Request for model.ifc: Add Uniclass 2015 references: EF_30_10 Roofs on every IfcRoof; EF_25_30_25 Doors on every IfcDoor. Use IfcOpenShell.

First a look at what the model holds.

```python
import ifcopenshell

model = ifcopenshell.open("model.ifc")
print(model.schema)
print("classifications:", [c.Name for c in model.by_type("IfcClassification")])
for ifc_class in ("IfcDoor", "IfcRoof", "IfcStair", "IfcWall", "IfcWindow"):
    print(ifc_class, len(model.by_type(ifc_class)))
```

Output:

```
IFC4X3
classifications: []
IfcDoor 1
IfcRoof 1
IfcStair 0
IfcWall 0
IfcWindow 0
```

```python
import ifcopenshell
import ifcopenshell.api.classification

model = ifcopenshell.open("model.ifc")

system = ifcopenshell.api.classification.add_classification(model, classification="Uniclass 2015")

codes = {
    "IfcRoof": ("EF_30_10", "Roofs"),
    "IfcDoor": ("EF_25_30_25", "Doors"),
}
for ifc_class, (code, name) in codes.items():
    products = model.by_type(ifc_class)
    ifcopenshell.api.classification.add_reference(
        model, products=products, classification=system, identification=code, name=name
    )
    print(code, len(products))

model.write("model_v2.ifc")
```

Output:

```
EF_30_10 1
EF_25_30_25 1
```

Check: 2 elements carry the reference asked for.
